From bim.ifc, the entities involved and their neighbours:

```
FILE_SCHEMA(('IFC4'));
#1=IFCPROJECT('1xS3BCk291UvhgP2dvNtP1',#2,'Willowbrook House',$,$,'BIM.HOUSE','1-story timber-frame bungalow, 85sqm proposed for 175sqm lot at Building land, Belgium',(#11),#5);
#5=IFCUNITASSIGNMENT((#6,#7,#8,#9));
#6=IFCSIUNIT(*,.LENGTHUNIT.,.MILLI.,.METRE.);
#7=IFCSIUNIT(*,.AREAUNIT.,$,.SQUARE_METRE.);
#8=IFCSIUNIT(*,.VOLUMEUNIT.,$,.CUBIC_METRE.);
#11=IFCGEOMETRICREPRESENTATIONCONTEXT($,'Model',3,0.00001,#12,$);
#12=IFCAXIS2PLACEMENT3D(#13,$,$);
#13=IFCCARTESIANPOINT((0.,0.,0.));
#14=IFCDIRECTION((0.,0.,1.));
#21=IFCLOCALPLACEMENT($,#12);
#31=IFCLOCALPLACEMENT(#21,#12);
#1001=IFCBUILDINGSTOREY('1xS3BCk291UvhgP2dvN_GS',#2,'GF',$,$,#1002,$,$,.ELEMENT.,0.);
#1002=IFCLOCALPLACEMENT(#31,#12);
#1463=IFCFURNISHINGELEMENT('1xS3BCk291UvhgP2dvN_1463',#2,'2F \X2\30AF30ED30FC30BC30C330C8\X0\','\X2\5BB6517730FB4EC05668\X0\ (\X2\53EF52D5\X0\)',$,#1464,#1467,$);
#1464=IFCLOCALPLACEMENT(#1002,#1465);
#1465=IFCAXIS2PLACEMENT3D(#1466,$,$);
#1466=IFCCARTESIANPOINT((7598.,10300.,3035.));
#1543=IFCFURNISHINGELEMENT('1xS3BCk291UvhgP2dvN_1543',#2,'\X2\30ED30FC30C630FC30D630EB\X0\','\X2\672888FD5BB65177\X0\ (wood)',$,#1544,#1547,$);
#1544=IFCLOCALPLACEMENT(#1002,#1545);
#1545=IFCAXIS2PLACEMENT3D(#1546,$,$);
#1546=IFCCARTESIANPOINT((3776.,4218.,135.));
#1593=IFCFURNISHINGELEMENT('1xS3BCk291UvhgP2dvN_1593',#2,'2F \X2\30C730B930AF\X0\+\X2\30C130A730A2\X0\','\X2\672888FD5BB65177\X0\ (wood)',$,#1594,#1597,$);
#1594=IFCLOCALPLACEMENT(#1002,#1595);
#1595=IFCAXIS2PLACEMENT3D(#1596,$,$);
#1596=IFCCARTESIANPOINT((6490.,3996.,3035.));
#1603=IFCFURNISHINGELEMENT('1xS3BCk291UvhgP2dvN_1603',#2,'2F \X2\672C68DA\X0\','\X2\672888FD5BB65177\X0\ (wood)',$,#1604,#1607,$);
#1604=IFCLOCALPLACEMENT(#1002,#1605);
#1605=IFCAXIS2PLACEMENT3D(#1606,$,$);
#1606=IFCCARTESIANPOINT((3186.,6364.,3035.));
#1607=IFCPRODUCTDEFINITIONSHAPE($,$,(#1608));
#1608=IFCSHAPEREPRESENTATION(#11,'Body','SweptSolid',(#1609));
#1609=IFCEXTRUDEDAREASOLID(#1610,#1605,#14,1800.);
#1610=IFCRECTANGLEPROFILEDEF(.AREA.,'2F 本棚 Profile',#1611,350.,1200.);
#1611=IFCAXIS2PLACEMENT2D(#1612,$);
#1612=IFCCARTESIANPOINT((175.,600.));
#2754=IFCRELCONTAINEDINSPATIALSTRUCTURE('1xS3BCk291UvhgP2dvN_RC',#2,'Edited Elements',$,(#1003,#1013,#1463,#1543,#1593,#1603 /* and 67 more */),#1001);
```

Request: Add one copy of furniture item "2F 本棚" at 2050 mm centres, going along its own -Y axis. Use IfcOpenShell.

```python
import ifcopenshell
import ifcopenshell.api.geometry
import ifcopenshell.api.root
import ifcopenshell.util.element
import ifcopenshell.util.placement
import ifcopenshell.util.unit

model = ifcopenshell.open("bim.ifc")
unit_scale = ifcopenshell.util.unit.calculate_unit_scale(model)


def reuse_history(source, copy):
    """copy_class also copies each property set's owner history, people and application; keep the originals."""
    for rel in copy.IsDefinedBy:
        if rel.is_a("IfcRelDefinesByProperties") and (history := rel.RelatingPropertyDefinition.OwnerHistory):
            rel.RelatingPropertyDefinition.OwnerHistory = source.OwnerHistory
            ifcopenshell.util.element.remove_deep2(model, history)


source = model.by_id(1603)
base = ifcopenshell.util.placement.get_local_placement(source.ObjectPlacement)
step = -base[:3, 1] * 2.05 / unit_scale

for i in range(1, 2):
    copy = ifcopenshell.api.root.copy_class(model, product=source)
    copy.Representation = ifcopenshell.util.element.copy_deep(
        model, source.Representation, exclude=["IfcGeometricRepresentationContext", "IfcRepresentationMap"]
    )
    reuse_history(source, copy)
    matrix = base.copy()
    matrix[:3, 3] += i * step
    print("added at", matrix[:3, 3].round(3) + 0.0)
    ifcopenshell.api.geometry.edit_object_placement(model, product=copy, matrix=matrix, is_si=False)

model.write("bim_rev.ifc")
```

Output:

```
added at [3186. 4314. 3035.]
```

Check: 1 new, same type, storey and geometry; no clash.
